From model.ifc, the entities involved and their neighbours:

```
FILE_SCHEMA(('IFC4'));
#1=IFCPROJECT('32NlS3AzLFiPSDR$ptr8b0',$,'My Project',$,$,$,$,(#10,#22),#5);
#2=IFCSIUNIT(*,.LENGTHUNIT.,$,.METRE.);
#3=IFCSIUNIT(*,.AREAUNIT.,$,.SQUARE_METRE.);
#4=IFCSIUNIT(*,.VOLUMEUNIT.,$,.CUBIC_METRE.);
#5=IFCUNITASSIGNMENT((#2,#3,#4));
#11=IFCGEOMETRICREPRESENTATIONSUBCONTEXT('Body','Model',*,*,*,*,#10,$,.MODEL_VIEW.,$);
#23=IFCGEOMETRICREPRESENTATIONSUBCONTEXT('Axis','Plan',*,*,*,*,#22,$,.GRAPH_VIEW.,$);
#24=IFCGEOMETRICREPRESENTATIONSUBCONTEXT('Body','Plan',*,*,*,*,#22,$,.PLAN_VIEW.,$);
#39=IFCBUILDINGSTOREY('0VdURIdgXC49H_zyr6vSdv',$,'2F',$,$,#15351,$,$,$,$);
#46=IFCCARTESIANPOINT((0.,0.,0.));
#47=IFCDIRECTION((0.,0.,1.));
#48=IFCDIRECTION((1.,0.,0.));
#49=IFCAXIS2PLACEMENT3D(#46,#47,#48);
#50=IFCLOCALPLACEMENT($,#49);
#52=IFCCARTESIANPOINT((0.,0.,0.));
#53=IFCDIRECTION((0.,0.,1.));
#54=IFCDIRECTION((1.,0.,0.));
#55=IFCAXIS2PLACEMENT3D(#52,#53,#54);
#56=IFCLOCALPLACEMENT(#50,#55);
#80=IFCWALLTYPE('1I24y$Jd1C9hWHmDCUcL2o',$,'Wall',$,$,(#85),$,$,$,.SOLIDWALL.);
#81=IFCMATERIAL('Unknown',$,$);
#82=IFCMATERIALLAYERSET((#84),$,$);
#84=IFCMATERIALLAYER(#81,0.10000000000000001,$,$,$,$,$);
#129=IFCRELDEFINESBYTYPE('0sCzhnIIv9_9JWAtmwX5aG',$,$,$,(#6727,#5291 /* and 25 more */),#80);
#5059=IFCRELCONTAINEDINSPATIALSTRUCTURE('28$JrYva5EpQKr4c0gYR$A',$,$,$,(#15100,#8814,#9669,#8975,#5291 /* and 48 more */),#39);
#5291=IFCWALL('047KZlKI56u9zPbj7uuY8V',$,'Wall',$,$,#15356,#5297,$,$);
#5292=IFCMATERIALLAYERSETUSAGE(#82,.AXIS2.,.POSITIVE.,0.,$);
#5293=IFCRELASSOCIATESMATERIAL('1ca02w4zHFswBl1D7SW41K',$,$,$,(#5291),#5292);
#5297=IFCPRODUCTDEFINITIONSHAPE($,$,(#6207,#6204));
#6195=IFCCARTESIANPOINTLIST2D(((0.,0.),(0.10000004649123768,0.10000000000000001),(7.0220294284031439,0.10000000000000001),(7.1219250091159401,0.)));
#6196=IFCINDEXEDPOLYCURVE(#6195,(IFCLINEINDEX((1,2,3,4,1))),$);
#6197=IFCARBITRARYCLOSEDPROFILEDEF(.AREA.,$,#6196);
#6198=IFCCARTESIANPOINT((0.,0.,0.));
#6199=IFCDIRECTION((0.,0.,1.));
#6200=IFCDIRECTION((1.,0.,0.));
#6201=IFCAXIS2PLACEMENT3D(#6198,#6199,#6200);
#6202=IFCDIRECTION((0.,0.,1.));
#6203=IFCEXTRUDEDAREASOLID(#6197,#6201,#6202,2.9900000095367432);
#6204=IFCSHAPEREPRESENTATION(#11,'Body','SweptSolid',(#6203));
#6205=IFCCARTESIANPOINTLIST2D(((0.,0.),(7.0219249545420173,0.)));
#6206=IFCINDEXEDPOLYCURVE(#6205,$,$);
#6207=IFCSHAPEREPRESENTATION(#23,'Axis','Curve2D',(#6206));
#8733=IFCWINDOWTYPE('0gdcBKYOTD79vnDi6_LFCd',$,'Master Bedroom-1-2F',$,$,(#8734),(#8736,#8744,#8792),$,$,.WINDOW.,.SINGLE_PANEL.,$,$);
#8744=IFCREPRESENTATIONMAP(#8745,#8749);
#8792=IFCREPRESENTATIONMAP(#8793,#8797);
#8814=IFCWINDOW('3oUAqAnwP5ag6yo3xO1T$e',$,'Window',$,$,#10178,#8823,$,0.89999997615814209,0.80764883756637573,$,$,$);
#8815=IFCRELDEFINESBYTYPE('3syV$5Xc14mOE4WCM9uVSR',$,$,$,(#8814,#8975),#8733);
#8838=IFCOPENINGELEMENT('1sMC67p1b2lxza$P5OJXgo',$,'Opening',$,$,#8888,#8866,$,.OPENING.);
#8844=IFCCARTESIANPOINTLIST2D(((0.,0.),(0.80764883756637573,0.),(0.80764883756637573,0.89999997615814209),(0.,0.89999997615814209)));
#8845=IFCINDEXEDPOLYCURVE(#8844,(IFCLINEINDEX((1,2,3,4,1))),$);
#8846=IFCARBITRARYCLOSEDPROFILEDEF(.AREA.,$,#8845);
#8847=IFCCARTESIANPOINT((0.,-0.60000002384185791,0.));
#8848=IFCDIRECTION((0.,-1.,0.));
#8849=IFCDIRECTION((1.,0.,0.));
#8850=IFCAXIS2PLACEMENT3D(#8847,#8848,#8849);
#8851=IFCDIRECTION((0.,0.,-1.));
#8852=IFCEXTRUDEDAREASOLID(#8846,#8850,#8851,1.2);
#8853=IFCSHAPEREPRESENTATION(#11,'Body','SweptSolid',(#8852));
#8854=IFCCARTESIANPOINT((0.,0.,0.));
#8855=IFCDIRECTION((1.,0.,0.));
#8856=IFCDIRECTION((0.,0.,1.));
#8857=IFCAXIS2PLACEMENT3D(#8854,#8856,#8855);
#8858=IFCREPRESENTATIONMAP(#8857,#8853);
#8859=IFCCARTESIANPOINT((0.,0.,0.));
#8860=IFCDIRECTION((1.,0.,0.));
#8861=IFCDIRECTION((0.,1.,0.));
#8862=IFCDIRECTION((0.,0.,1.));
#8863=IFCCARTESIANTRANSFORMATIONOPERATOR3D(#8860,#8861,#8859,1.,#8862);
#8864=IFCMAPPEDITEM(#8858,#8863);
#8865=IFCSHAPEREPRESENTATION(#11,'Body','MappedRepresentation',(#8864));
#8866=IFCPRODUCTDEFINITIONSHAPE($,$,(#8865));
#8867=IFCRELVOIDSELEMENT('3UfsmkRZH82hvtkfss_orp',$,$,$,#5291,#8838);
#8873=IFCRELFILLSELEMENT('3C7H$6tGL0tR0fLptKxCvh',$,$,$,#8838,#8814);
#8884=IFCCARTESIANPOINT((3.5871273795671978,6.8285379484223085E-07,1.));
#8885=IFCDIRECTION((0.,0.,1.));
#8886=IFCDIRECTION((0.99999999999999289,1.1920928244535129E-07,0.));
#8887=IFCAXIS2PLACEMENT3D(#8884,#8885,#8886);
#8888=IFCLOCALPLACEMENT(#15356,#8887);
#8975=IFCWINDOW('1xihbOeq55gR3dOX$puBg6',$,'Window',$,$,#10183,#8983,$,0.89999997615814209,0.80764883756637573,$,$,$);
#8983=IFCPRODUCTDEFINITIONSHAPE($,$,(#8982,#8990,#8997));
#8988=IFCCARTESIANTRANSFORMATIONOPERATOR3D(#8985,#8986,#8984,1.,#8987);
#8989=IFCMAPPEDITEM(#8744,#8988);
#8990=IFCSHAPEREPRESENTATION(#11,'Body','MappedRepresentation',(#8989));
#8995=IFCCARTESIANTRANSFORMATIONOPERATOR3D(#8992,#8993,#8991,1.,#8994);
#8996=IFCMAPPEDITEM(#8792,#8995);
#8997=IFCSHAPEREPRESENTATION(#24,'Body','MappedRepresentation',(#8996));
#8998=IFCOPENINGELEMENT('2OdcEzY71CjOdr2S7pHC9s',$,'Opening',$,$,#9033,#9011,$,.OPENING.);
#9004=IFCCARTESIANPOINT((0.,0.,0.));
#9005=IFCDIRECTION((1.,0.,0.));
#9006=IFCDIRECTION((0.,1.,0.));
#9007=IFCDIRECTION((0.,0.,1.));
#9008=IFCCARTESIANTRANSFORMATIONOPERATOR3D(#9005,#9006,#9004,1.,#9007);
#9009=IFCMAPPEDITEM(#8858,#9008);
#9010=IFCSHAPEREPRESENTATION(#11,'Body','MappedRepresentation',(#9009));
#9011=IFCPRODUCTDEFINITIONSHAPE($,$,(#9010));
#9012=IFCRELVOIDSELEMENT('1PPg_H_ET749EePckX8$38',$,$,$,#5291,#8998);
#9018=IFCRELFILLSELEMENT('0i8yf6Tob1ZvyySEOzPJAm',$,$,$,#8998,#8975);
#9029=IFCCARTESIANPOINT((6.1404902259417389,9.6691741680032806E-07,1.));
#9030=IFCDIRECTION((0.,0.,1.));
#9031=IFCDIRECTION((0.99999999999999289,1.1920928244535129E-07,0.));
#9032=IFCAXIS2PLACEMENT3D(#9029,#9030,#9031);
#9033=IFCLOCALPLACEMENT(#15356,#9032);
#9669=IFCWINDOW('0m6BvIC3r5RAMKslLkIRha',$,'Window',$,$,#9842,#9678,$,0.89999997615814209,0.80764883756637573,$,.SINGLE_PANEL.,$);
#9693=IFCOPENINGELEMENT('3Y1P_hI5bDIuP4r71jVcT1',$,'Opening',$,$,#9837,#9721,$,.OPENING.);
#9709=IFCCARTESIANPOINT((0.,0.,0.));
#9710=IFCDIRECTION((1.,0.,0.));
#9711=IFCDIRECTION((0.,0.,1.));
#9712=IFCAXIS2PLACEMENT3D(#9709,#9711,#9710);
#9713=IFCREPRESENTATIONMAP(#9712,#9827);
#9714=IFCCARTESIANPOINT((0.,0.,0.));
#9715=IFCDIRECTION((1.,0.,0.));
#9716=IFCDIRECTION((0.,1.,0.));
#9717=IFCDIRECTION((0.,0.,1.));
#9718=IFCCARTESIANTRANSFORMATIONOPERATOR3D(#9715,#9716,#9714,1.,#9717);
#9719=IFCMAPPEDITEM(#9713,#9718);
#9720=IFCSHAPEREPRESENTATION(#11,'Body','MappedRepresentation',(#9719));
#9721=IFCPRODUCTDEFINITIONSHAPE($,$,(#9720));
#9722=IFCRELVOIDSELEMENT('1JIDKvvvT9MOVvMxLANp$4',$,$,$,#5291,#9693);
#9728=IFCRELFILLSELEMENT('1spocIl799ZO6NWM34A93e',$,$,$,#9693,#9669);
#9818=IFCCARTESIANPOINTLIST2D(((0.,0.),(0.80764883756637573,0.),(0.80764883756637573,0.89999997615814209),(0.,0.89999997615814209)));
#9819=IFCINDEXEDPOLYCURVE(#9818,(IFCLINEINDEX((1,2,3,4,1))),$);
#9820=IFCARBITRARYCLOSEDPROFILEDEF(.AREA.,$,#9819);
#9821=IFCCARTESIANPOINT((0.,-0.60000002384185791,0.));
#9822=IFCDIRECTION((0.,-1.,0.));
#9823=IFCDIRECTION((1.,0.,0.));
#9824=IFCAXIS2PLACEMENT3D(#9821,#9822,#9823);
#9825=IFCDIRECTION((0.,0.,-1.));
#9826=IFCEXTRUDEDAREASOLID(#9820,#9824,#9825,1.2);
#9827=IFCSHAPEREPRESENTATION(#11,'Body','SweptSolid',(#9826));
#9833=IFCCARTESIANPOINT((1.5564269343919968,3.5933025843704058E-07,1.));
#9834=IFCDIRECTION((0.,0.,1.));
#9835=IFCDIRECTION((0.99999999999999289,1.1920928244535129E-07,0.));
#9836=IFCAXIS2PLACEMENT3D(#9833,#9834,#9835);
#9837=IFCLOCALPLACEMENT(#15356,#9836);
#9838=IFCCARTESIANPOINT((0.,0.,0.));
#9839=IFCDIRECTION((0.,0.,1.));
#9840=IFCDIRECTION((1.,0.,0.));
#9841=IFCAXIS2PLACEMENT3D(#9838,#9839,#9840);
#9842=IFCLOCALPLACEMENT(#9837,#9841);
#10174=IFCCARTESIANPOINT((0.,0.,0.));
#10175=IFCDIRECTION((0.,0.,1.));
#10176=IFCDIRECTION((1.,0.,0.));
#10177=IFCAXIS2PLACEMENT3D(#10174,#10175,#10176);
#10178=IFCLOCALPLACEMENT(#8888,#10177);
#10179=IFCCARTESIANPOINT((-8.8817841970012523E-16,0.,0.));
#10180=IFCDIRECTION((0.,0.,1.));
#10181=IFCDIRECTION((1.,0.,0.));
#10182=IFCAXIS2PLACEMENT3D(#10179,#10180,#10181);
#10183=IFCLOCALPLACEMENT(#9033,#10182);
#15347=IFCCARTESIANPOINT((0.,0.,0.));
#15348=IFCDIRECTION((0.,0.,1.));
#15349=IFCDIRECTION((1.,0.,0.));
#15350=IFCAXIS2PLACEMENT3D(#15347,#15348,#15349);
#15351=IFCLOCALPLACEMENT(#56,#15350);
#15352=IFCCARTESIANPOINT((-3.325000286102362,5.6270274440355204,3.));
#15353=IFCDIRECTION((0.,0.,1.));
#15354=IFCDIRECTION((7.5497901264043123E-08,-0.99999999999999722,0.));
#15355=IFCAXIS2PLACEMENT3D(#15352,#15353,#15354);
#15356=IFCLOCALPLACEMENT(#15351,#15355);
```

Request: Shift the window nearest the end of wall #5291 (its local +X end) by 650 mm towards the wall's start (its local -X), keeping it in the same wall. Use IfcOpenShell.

```python
import ifcopenshell
import ifcopenshell.api.geometry
import ifcopenshell.util.placement

model = ifcopenshell.open("model.ifc")

window = model.by_id(8975)
opening = window.FillsVoids[0].RelatingOpeningElement
wall = opening.VoidsElements[0].RelatingBuildingElement

wall_matrix = ifcopenshell.util.placement.get_local_placement(wall.ObjectPlacement)
shift = wall_matrix[:3, 0] * -0.65
before = ifcopenshell.util.placement.get_local_placement(window.ObjectPlacement)[:3, 3].copy()

# The window is placed relative to its opening, so it follows when the opening moves.
matrix = ifcopenshell.util.placement.get_local_placement(opening.ObjectPlacement)
matrix[:3, 3] += shift
ifcopenshell.api.geometry.edit_object_placement(
    model, product=opening, matrix=matrix, is_si=False, should_transform_children=True
)

after = ifcopenshell.util.placement.get_local_placement(window.ObjectPlacement)[:3, 3]
print("window moved by", (after - before).round(3) + 0.0)

model.write("model_edited.ifc")
```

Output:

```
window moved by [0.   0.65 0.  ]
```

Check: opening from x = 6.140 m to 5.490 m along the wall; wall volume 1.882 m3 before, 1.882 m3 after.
